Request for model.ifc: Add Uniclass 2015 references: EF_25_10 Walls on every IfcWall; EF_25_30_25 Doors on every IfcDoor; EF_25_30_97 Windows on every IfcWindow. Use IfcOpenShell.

First a look at what the model holds.

```python
import ifcopenshell

model = ifcopenshell.open("model.ifc")
print(model.schema)
print("classifications:", [c.Name for c in model.by_type("IfcClassification")])
for ifc_class in ("IfcDoor", "IfcRoof", "IfcStair", "IfcWall", "IfcWindow"):
    print(ifc_class, len(model.by_type(ifc_class)))
```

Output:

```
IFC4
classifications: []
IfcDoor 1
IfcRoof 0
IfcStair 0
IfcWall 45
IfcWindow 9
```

```python
import ifcopenshell
import ifcopenshell.api.classification

model = ifcopenshell.open("model.ifc")

system = ifcopenshell.api.classification.add_classification(model, classification="Uniclass 2015")

codes = {
    "IfcWall": ("EF_25_10", "Walls"),
    "IfcDoor": ("EF_25_30_25", "Doors"),
    "IfcWindow": ("EF_25_30_97", "Windows"),
}
for ifc_class, (code, name) in codes.items():
    products = model.by_type(ifc_class)
    ifcopenshell.api.classification.add_reference(
        model, products=products, classification=system, identification=code, name=name
    )
    print(code, len(products))

model.write("model_edited.ifc")
```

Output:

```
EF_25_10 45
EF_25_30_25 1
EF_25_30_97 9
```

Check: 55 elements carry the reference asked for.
